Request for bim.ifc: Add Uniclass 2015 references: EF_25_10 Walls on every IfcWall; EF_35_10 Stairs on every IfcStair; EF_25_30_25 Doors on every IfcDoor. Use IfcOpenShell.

First a look at what the model holds.

```python
import ifcopenshell

model = ifcopenshell.open("bim.ifc")
print(model.schema)
print("classifications:", [c.Name for c in model.by_type("IfcClassification")])
for ifc_class in ("IfcDoor", "IfcRoof", "IfcStair", "IfcWall", "IfcWindow"):
    print(ifc_class, len(model.by_type(ifc_class)))
```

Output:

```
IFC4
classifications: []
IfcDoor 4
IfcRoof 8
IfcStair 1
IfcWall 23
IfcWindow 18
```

```python
import ifcopenshell
import ifcopenshell.api.classification

model = ifcopenshell.open("bim.ifc")

system = ifcopenshell.api.classification.add_classification(model, classification="Uniclass 2015")

codes = {
    "IfcWall": ("EF_25_10", "Walls"),
    "IfcStair": ("EF_35_10", "Stairs"),
    "IfcDoor": ("EF_25_30_25", "Doors"),
}
for ifc_class, (code, name) in codes.items():
    products = model.by_type(ifc_class)
    ifcopenshell.api.classification.add_reference(
        model, products=products, classification=system, identification=code, name=name
    )
    print(code, len(products))

model.write("bim_rev.ifc")
```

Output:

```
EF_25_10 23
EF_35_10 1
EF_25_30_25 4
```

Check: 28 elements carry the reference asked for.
